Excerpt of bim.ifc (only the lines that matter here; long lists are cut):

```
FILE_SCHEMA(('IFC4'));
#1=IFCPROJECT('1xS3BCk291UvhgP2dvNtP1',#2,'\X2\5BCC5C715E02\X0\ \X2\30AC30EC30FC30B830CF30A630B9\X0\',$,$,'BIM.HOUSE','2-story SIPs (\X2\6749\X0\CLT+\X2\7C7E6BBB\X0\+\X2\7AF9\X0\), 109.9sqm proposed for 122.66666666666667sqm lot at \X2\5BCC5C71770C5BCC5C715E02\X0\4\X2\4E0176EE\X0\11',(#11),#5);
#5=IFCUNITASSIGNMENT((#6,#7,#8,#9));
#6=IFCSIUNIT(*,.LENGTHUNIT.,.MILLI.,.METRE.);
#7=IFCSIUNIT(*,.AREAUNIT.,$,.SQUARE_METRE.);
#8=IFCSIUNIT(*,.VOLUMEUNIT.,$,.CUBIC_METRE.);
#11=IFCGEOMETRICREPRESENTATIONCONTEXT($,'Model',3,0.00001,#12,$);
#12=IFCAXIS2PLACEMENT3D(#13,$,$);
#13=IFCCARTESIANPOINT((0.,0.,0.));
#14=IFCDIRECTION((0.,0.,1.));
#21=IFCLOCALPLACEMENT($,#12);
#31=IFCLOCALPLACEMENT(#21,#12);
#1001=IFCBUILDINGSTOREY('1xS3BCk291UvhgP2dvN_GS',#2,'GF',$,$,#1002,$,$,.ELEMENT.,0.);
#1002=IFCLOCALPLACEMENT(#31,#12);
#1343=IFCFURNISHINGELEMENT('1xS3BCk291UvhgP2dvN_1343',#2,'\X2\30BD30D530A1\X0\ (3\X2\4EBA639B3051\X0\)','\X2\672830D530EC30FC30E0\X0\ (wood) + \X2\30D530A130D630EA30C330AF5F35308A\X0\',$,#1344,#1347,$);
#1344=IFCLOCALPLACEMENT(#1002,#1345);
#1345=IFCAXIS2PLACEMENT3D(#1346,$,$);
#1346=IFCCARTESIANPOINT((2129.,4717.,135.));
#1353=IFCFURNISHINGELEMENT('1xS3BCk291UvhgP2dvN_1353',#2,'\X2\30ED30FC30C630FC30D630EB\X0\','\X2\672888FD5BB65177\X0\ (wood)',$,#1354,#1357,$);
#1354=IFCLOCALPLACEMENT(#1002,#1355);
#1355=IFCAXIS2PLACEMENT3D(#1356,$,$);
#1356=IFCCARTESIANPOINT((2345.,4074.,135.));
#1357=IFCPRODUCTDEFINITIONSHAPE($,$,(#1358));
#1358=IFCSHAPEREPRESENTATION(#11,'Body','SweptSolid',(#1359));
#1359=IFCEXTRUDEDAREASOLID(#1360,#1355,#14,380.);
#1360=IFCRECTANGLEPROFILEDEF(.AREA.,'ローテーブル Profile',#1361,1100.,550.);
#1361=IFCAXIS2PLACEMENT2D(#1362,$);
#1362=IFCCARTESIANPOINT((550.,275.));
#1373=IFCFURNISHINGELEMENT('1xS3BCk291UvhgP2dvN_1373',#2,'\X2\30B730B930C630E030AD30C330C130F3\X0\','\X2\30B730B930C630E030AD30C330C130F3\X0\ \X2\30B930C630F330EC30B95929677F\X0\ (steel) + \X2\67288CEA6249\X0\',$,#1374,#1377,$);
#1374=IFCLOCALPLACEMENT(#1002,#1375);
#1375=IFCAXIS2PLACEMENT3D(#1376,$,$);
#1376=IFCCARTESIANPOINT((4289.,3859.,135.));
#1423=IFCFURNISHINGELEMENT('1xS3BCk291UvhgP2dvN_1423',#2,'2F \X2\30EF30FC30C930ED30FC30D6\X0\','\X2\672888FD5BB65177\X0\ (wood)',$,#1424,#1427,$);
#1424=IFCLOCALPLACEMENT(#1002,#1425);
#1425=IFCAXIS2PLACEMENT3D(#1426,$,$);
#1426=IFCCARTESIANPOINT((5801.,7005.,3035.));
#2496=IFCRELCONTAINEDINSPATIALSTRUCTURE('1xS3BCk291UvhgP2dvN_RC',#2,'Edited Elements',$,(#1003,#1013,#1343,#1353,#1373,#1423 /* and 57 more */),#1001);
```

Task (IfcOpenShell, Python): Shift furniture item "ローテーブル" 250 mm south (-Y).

```python
import ifcopenshell
import ifcopenshell.api.geometry
import ifcopenshell.util.placement
import ifcopenshell.util.unit

model = ifcopenshell.open("bim.ifc")
unit_scale = ifcopenshell.util.unit.calculate_unit_scale(model)

item = model.by_guid("1xS3BCk291UvhgP2dvN_1353")
matrix = ifcopenshell.util.placement.get_local_placement(item.ObjectPlacement)
matrix[1, 3] -= 0.25 / unit_scale
ifcopenshell.api.geometry.edit_object_placement(model, product=item, matrix=matrix, is_si=False)

print(ifcopenshell.util.placement.get_local_placement(item.ObjectPlacement).round(3) + 0.0)

model.write("bim_v2.ifc")
```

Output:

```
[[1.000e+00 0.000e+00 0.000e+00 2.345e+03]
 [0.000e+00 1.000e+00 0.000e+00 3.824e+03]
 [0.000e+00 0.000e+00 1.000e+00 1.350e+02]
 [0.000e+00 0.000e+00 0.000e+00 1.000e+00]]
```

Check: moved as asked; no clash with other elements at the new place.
